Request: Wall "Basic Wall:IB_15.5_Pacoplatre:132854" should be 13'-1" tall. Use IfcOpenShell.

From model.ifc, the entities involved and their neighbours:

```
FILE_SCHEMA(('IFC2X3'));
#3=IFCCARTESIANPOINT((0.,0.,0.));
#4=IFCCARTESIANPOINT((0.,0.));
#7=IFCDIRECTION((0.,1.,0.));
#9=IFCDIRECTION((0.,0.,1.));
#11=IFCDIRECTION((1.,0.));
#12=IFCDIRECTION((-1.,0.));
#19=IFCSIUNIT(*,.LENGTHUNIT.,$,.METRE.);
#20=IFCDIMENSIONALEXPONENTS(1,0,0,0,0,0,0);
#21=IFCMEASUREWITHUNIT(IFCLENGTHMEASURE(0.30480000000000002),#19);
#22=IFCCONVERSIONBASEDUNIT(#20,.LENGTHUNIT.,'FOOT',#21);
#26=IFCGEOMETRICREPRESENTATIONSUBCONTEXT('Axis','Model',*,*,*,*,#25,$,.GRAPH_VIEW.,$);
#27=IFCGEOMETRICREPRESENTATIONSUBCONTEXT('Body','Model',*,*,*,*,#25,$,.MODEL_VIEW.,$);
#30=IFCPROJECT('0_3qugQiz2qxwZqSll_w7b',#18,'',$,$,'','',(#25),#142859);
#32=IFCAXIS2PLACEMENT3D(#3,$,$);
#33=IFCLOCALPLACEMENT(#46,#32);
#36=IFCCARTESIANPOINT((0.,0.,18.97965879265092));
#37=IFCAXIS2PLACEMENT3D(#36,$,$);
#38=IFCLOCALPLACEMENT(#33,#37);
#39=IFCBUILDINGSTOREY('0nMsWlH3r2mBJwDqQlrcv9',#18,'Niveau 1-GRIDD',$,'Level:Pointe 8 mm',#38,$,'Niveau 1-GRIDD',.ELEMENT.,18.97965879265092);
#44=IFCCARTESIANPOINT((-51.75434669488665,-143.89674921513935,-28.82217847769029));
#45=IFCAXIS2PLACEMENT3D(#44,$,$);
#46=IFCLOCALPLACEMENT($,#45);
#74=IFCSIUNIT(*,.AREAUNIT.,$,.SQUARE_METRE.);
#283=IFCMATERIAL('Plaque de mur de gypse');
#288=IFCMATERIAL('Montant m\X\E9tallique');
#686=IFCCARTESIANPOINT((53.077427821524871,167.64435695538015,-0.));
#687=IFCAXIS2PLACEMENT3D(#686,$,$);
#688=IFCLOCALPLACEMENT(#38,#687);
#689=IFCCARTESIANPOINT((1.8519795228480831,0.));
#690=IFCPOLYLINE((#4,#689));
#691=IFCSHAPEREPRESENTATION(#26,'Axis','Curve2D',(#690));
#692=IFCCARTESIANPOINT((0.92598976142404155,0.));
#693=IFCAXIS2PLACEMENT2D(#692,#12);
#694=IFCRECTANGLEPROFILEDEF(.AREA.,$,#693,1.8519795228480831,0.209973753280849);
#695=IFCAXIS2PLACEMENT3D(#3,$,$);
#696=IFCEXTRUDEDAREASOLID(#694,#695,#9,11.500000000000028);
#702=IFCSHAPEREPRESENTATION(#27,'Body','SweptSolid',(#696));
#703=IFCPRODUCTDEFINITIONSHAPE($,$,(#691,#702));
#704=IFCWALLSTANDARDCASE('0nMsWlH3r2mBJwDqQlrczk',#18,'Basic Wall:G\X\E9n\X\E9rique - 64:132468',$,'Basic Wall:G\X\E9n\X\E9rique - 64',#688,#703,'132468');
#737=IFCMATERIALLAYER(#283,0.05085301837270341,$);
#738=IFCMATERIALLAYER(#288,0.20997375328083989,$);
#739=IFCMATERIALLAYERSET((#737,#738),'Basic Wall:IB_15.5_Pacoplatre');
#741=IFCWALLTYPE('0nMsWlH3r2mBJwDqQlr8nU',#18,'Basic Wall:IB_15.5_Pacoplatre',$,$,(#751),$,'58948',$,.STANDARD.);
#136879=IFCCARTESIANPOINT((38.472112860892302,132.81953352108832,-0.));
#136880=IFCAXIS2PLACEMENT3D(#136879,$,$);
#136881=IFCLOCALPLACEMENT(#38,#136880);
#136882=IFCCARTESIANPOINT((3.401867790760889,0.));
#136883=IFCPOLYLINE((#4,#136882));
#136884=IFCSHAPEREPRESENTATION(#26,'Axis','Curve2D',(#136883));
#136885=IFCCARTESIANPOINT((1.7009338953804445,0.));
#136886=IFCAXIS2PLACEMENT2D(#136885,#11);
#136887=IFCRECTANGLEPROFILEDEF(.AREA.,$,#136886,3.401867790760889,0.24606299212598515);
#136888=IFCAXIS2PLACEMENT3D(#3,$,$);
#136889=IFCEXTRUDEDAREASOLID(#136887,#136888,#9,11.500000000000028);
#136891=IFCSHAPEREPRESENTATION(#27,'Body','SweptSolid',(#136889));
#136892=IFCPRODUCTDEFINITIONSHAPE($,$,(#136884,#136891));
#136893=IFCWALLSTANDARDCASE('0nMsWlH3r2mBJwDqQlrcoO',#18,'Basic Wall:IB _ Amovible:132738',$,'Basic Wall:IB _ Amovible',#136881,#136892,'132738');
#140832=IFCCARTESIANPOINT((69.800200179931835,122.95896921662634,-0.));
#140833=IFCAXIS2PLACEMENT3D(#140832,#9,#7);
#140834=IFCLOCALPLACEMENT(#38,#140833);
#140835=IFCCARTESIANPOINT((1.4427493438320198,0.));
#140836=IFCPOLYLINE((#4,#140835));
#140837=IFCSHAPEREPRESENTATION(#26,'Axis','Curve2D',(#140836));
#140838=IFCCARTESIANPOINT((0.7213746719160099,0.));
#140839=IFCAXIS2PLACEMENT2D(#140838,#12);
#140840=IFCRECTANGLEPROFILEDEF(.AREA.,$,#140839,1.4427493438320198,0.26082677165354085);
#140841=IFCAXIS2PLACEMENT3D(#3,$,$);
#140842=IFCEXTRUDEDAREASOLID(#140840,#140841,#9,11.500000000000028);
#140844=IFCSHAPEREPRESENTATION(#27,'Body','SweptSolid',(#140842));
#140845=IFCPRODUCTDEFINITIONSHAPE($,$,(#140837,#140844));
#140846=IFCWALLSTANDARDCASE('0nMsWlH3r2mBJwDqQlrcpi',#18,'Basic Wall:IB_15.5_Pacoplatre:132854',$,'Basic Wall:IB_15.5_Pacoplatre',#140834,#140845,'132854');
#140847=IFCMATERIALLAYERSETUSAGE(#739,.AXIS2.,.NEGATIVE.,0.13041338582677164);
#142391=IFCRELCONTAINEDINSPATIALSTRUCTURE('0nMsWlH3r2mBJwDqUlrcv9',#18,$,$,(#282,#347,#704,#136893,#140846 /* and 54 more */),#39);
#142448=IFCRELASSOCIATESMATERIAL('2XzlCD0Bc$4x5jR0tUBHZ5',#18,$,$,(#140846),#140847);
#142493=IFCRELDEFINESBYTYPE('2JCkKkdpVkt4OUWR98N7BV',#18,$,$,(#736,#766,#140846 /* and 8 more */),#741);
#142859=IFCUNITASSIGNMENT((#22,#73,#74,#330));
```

```python
import ifcopenshell
import ifcopenshell.geom
import ifcopenshell.util.representation
import ifcopenshell.util.shape
import ifcopenshell.util.unit

model = ifcopenshell.open("model.ifc")
unit_scale = ifcopenshell.util.unit.calculate_unit_scale(model)
settings = ifcopenshell.geom.settings()


def volume(element):
    """Net volume in cubic metres, openings subtracted."""
    shape = ifcopenshell.geom.create_shape(settings, element)
    return ifcopenshell.util.shape.get_volume(shape.geometry)


wall = model.by_guid("0nMsWlH3r2mBJwDqQlrcpi")
before = volume(wall)

body = ifcopenshell.util.representation.get_representation(wall, "Model", "Body")
solid = body.Items[0]
old_height = solid.Depth
solid.Depth = 157 * 0.0254 / unit_scale
after = volume(wall)

print(f"height {old_height:g} -> {solid.Depth:g}, volume {before:.3f} -> {after:.3f} m3")

model.write("model_rev.ifc")
```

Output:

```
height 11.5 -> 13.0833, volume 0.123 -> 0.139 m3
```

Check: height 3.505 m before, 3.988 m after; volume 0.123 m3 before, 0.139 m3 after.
